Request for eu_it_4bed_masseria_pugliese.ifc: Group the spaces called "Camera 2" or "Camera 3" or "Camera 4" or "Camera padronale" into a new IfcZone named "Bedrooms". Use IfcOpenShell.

First a look at what the model holds.

```python
import ifcopenshell

model = ifcopenshell.open("eu_it_4bed_masseria_pugliese.ifc")
print(model.schema)
seen = {}
for space in model.by_type("IfcSpace"):
    seen[space.LongName] = seen.get(space.LongName, 0) + 1
for name, count in sorted(seen.items(), key=str):
    print(count, "x", name)
print("zones:", [z.Name for z in model.by_type("IfcZone")][:20])
```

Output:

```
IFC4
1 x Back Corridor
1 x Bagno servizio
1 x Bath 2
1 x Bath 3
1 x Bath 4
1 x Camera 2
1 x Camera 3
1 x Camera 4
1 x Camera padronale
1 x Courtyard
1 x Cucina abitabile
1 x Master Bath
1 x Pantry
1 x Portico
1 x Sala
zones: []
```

```python
import ifcopenshell
import ifcopenshell.api.group
import ifcopenshell.api.root

model = ifcopenshell.open("eu_it_4bed_masseria_pugliese.ifc")

names = {"Camera 2", "Camera 3", "Camera 4", "Camera padronale"}
spaces = [s for s in model.by_type("IfcSpace") if s.LongName in names]

zone = ifcopenshell.api.root.create_entity(model, ifc_class="IfcZone", name="Bedrooms")
ifcopenshell.api.group.assign_group(model, products=spaces, group=zone)
print(len(spaces), "spaces in", zone.Name)

model.write("eu_it_4bed_masseria_pugliese_updated.ifc")
```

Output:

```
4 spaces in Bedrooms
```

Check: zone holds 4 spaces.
